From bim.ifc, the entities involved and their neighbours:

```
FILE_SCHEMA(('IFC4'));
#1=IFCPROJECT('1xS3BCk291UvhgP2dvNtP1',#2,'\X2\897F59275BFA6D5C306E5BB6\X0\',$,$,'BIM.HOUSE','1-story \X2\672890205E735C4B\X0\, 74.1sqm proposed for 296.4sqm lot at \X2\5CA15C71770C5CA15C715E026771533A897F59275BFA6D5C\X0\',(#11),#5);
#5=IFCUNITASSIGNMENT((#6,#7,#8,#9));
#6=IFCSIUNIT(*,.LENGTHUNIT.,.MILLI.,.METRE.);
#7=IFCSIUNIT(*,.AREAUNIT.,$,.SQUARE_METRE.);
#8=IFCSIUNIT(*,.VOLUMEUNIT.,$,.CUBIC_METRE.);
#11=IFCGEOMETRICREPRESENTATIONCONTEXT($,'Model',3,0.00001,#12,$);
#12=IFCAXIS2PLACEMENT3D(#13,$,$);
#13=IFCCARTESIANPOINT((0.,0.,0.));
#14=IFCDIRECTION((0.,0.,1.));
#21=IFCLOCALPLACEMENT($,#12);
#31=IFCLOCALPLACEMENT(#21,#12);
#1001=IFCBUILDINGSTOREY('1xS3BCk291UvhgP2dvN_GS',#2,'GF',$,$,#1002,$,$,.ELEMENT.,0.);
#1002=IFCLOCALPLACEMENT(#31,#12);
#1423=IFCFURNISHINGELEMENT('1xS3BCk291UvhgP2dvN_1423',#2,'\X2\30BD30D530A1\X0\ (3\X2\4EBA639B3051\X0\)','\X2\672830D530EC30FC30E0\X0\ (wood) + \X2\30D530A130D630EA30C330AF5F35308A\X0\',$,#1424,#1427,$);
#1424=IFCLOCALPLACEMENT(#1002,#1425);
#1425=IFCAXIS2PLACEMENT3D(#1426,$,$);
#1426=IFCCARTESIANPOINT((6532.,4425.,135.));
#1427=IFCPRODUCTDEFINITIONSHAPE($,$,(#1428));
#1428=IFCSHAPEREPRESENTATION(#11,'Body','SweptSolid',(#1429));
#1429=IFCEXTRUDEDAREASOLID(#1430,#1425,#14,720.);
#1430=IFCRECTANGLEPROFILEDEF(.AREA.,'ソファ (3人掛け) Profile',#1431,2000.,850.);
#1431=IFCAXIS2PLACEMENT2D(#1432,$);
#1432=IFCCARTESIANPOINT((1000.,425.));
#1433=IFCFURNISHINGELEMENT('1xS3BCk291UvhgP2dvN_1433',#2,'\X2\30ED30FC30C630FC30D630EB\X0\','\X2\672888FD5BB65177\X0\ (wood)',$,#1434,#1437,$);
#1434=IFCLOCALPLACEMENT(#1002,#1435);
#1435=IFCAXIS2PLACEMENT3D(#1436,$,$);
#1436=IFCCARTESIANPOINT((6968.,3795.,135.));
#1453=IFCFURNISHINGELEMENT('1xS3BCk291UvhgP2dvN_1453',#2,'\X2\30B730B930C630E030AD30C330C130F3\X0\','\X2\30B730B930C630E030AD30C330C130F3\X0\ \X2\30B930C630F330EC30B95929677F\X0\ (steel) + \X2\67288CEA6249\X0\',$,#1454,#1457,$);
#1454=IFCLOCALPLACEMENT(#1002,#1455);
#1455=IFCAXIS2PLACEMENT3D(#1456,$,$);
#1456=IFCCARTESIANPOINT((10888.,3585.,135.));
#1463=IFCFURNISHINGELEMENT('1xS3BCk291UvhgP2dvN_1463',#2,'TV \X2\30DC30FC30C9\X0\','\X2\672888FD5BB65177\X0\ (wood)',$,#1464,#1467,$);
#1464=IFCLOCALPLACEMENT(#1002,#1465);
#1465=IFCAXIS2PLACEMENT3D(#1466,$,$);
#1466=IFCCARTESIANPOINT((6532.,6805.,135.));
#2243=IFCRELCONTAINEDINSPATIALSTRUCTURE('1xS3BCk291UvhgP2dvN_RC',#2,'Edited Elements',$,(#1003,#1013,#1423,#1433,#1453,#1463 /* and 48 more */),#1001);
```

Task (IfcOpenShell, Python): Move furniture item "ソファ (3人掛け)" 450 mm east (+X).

```python
import ifcopenshell
import ifcopenshell.api.geometry
import ifcopenshell.util.placement
import ifcopenshell.util.unit

model = ifcopenshell.open("bim.ifc")
unit_scale = ifcopenshell.util.unit.calculate_unit_scale(model)

item = model.by_guid("1xS3BCk291UvhgP2dvN_1423")
matrix = ifcopenshell.util.placement.get_local_placement(item.ObjectPlacement)
matrix[0, 3] += 0.45 / unit_scale
ifcopenshell.api.geometry.edit_object_placement(model, product=item, matrix=matrix, is_si=False)

print(ifcopenshell.util.placement.get_local_placement(item.ObjectPlacement).round(3) + 0.0)

model.write("bim_rev.ifc")
```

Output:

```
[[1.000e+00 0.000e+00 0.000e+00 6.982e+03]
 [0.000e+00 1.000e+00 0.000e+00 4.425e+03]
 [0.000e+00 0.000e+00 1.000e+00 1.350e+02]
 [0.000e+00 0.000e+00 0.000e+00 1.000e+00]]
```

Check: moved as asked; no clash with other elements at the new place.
